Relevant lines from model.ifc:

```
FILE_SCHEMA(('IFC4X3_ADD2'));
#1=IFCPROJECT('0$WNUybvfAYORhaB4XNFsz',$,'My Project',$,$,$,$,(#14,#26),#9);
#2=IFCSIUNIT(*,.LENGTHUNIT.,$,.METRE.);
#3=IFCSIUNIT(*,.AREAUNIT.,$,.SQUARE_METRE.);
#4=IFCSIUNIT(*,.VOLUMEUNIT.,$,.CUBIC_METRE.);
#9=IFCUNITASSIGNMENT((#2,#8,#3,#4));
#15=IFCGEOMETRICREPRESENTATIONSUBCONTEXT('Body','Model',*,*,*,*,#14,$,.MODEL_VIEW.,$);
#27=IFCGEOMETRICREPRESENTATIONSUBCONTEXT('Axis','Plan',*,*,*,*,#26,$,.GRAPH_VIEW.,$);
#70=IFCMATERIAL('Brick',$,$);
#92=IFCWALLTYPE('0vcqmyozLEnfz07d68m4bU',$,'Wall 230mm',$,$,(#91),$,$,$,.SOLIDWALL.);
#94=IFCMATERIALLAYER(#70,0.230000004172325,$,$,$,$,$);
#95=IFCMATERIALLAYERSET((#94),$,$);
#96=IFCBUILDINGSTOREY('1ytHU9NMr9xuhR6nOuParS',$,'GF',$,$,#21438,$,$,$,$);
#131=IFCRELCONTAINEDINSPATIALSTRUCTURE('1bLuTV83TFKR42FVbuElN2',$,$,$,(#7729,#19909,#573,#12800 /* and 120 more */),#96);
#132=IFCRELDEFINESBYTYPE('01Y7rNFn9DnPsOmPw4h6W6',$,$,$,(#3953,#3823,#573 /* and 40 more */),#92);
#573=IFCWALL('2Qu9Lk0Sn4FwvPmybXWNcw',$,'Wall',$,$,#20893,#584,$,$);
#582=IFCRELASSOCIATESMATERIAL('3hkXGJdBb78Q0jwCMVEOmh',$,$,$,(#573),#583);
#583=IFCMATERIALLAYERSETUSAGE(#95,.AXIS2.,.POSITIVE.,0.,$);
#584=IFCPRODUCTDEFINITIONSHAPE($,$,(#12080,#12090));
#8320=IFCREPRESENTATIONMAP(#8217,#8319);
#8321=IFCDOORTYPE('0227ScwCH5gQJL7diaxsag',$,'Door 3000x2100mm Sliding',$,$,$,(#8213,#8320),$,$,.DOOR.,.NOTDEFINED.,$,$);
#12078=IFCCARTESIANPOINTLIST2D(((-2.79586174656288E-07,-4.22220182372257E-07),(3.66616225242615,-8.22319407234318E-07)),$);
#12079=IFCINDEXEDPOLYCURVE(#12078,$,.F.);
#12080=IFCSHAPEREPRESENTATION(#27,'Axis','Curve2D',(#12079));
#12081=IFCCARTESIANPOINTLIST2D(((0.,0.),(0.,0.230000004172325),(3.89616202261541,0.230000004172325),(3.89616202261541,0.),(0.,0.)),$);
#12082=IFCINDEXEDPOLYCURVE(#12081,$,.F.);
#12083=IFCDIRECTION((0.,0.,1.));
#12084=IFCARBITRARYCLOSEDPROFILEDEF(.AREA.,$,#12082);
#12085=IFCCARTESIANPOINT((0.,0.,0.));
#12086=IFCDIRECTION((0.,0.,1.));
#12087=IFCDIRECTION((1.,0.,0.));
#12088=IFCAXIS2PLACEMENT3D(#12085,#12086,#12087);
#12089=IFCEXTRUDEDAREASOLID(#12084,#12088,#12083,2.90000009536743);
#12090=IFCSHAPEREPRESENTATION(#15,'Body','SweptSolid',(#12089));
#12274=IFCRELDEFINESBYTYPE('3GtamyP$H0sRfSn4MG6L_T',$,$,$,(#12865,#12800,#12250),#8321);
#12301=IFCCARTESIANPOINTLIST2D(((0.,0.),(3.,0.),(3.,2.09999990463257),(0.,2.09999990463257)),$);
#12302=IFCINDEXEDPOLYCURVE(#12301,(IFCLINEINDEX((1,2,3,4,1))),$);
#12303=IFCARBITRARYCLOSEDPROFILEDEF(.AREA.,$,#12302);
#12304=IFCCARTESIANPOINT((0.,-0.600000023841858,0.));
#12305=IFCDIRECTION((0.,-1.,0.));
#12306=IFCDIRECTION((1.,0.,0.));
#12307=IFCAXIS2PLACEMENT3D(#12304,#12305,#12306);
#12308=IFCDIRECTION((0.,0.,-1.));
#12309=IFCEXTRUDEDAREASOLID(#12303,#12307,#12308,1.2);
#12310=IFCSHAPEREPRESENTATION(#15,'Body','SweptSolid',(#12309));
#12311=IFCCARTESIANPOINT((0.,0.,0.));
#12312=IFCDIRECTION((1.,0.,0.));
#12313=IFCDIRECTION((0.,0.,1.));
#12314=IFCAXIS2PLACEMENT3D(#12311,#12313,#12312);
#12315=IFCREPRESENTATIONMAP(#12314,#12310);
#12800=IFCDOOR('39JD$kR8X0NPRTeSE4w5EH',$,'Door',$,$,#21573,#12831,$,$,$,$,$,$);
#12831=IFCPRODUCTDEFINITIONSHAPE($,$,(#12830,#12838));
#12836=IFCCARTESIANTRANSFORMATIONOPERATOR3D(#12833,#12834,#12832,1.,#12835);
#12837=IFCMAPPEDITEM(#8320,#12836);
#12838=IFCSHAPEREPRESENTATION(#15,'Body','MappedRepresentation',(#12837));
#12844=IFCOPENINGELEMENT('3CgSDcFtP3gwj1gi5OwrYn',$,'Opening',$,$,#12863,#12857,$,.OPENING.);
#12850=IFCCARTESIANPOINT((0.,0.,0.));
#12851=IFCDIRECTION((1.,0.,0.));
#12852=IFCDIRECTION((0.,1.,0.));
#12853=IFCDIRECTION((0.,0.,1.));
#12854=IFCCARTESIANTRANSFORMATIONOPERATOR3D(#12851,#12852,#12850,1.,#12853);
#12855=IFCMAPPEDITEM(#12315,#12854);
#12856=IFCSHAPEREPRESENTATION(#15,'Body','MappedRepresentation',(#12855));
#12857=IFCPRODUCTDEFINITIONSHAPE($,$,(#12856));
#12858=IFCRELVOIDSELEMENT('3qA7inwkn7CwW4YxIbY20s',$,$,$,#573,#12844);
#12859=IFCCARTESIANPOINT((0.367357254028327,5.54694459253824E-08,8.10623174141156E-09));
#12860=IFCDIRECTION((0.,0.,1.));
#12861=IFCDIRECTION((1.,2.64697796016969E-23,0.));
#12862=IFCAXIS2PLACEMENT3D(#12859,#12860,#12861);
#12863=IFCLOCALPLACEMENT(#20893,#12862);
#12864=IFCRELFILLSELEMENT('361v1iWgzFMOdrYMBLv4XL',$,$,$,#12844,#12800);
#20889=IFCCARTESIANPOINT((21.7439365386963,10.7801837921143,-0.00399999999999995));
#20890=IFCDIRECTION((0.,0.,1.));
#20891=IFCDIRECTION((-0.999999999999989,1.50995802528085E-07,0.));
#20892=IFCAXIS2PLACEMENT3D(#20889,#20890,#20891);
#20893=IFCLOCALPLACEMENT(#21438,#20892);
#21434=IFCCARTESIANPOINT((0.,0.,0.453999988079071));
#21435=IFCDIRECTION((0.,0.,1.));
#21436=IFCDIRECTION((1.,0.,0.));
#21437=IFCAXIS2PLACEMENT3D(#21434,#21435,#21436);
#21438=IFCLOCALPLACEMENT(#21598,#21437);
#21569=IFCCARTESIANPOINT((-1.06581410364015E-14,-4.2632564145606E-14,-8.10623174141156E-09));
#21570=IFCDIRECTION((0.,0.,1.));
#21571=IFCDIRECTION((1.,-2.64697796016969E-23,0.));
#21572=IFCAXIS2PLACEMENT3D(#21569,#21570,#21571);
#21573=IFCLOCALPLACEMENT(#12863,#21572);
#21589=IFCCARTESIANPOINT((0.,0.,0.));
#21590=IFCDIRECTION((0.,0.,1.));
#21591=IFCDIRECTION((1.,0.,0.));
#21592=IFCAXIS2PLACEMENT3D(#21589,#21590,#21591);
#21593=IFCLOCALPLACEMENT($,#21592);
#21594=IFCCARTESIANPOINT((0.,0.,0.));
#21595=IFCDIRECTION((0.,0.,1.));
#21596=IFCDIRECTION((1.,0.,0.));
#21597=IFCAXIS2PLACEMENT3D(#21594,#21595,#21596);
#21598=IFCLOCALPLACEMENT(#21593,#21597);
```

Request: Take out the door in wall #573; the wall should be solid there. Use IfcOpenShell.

```python
import ifcopenshell
import ifcopenshell.api.feature
import ifcopenshell.api.root
import ifcopenshell.geom
import ifcopenshell.util.shape

model = ifcopenshell.open("model.ifc")
settings = ifcopenshell.geom.settings()


def volume(element):
    """Net volume in cubic metres, openings subtracted."""
    shape = ifcopenshell.geom.create_shape(settings, element)
    return ifcopenshell.util.shape.get_volume(shape.geometry)


door = model.by_id(12800)
opening = door.FillsVoids[0].RelatingOpeningElement
wall = opening.VoidsElements[0].RelatingBuildingElement
before = volume(wall)

ifcopenshell.api.root.remove_product(model, product=door)
ifcopenshell.api.feature.remove_feature(model, feature=opening)

after = volume(wall)

print(f"wall volume {before:.3f} -> {after:.3f} m3")

model.write("model_updated.ifc")
```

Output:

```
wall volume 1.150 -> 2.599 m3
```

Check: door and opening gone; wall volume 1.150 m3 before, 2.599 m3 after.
